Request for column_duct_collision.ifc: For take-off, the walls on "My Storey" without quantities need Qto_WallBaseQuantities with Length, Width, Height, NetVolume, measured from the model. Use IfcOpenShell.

First a look at what the model holds.

```python
import ifcopenshell
import ifcopenshell.util.element
import ifcopenshell.util.unit

model = ifcopenshell.open("column_duct_collision.ifc")
print(model.schema)
for unit_type in ("LENGTHUNIT", "AREAUNIT", "VOLUMEUNIT"):
    print(unit_type, ifcopenshell.util.unit.calculate_unit_scale(model, unit_type))
storey = next(s for s in model.by_type("IfcBuildingStorey") if s.Name == "My Storey")
walls = [e for e in ifcopenshell.util.element.get_decomposition(storey) if e.is_a("IfcWall")]
for e in sorted(walls, key=lambda e: e.id()):
    print(e.id(), e.is_a(), e.Name, list(ifcopenshell.util.element.get_psets(e, qtos_only=True)), sep=" | ")
```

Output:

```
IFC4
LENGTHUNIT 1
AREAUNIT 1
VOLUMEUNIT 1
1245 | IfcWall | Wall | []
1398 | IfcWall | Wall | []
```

```python
import ifcopenshell
import ifcopenshell.api.pset
import ifcopenshell.geom
import ifcopenshell.util.element
import ifcopenshell.util.shape
import ifcopenshell.util.unit

model = ifcopenshell.open("column_duct_collision.ifc")
unit_scale = ifcopenshell.util.unit.calculate_unit_scale(model)
volume_scale = ifcopenshell.util.unit.calculate_unit_scale(model, "VOLUMEUNIT")
settings = ifcopenshell.geom.settings()

storey = next(s for s in model.by_type("IfcBuildingStorey") if s.Name == "My Storey")
walls = [e for e in ifcopenshell.util.element.get_decomposition(storey) if e.is_a("IfcWall")]

for e in sorted(walls, key=lambda e: e.id()):
    if ifcopenshell.util.element.get_psets(e, qtos_only=True, should_inherit=False):
        continue
    # Geometry comes back in metres, in the element's own axes.
    shape = ifcopenshell.geom.create_shape(settings, e)
    values = {
        "Length": ifcopenshell.util.shape.get_x(shape.geometry) / unit_scale,
        "Width": ifcopenshell.util.shape.get_y(shape.geometry) / unit_scale,
        "Height": ifcopenshell.util.shape.get_z(shape.geometry) / unit_scale,
        "NetVolume": ifcopenshell.util.shape.get_volume(shape.geometry) / volume_scale,
    }
    qto = ifcopenshell.api.pset.add_qto(model, product=e, name="Qto_WallBaseQuantities")
    ifcopenshell.api.pset.edit_qto(model, qto=qto, properties=values)
    print(e.id(), {k: round(v, 3) for k, v in values.items()})

model.write("column_duct_collision-out.ifc")
```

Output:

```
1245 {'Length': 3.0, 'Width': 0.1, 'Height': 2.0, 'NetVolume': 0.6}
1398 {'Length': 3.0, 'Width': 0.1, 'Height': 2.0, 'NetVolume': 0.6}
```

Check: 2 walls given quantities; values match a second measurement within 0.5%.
